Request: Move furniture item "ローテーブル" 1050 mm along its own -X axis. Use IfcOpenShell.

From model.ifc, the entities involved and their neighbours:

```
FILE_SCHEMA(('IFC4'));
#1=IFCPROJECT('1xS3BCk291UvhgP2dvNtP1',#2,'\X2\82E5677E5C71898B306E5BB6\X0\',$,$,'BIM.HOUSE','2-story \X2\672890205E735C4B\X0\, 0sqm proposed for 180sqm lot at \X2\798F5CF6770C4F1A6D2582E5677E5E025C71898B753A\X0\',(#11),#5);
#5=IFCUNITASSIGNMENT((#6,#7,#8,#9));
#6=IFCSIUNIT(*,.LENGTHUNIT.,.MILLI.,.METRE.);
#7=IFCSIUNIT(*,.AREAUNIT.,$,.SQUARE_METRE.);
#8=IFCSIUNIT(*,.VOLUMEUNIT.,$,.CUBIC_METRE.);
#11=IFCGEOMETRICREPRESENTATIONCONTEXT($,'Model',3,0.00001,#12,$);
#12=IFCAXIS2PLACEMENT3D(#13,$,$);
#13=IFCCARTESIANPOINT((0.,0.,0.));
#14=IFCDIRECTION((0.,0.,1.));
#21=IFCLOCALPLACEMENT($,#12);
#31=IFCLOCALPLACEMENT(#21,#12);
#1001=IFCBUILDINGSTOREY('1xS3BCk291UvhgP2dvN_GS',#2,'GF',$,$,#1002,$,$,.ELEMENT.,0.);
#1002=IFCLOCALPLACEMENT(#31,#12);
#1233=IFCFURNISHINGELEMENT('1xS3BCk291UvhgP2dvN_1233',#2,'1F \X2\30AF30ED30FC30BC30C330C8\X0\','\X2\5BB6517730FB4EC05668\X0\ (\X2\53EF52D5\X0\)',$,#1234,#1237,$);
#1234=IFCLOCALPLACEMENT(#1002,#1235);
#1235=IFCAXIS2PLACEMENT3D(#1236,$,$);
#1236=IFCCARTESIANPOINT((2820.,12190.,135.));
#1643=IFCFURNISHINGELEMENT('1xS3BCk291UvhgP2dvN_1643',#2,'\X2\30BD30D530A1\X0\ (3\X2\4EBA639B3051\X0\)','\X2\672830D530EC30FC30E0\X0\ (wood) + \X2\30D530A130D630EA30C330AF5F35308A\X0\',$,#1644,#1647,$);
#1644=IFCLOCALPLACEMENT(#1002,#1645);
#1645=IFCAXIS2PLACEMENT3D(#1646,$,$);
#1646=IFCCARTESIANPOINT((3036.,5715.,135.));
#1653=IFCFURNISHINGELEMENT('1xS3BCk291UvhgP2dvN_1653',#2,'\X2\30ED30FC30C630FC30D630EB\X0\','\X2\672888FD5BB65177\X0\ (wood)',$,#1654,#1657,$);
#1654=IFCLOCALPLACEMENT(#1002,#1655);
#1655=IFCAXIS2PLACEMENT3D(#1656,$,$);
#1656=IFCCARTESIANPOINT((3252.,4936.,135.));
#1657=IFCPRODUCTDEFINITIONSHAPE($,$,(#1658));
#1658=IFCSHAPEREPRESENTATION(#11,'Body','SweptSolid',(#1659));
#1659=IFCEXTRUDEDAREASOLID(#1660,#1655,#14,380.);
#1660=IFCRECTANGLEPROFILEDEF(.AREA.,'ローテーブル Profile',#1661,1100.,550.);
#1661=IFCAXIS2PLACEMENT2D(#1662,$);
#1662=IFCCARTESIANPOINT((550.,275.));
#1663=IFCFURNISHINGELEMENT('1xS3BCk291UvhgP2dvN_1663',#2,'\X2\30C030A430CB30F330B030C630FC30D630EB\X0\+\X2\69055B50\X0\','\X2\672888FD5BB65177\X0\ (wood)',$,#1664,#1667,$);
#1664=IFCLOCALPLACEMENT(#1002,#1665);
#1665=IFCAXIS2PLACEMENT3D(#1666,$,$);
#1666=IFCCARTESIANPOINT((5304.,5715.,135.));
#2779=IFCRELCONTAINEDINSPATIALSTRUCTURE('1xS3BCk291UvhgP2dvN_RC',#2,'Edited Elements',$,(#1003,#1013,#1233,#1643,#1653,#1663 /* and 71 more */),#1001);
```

```python
import ifcopenshell
import ifcopenshell.api.geometry
import ifcopenshell.util.placement
import ifcopenshell.util.unit

model = ifcopenshell.open("model.ifc")
unit_scale = ifcopenshell.util.unit.calculate_unit_scale(model)

item = model.by_guid("1xS3BCk291UvhgP2dvN_1653")
matrix = ifcopenshell.util.placement.get_local_placement(item.ObjectPlacement)
matrix[:3, 3] -= matrix[:3, 0] * 1.05 / unit_scale
ifcopenshell.api.geometry.edit_object_placement(model, product=item, matrix=matrix, is_si=False)

print(ifcopenshell.util.placement.get_local_placement(item.ObjectPlacement).round(3) + 0.0)

model.write("model_edited.ifc")
```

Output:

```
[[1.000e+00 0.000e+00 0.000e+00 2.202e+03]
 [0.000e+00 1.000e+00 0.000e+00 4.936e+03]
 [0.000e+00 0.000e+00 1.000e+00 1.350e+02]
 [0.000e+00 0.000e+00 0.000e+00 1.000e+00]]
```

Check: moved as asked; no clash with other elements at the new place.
